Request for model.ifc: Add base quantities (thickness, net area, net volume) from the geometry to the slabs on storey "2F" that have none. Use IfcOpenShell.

First a look at what the model holds.

```python
import ifcopenshell
import ifcopenshell.util.element
import ifcopenshell.util.unit

model = ifcopenshell.open("model.ifc")
print(model.schema)
for unit_type in ("LENGTHUNIT", "AREAUNIT", "VOLUMEUNIT"):
    print(unit_type, ifcopenshell.util.unit.calculate_unit_scale(model, unit_type))
storey = next(s for s in model.by_type("IfcBuildingStorey") if s.Name == "2F")
slabs = [e for e in ifcopenshell.util.element.get_decomposition(storey) if e.is_a("IfcSlab")]
for e in sorted(slabs, key=lambda e: e.id()):
    print(e.id(), e.is_a(), e.Name, list(ifcopenshell.util.element.get_psets(e, qtos_only=True)), sep=" | ")
```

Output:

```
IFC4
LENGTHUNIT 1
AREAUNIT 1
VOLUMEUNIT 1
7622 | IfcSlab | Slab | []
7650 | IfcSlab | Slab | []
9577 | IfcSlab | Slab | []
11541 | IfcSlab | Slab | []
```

```python
import ifcopenshell
import ifcopenshell.api.pset
import ifcopenshell.geom
import ifcopenshell.util.element
import ifcopenshell.util.shape
import ifcopenshell.util.unit

model = ifcopenshell.open("model.ifc")
unit_scale = ifcopenshell.util.unit.calculate_unit_scale(model)
area_scale = ifcopenshell.util.unit.calculate_unit_scale(model, "AREAUNIT")
volume_scale = ifcopenshell.util.unit.calculate_unit_scale(model, "VOLUMEUNIT")
settings = ifcopenshell.geom.settings()

storey = next(s for s in model.by_type("IfcBuildingStorey") if s.Name == "2F")
slabs = [e for e in ifcopenshell.util.element.get_decomposition(storey) if e.is_a("IfcSlab")]

for e in sorted(slabs, key=lambda e: e.id()):
    if ifcopenshell.util.element.get_psets(e, qtos_only=True, should_inherit=False):
        continue
    # Geometry comes back in metres, in the element's own axes.
    shape = ifcopenshell.geom.create_shape(settings, e)
    values = {
        "Width": ifcopenshell.util.shape.get_z(shape.geometry) / unit_scale,
        "NetArea": ifcopenshell.util.shape.get_footprint_area(shape.geometry) / area_scale,
        "NetVolume": ifcopenshell.util.shape.get_volume(shape.geometry) / volume_scale,
    }
    qto = ifcopenshell.api.pset.add_qto(model, product=e, name="Qto_SlabBaseQuantities")
    ifcopenshell.api.pset.edit_qto(model, qto=qto, properties=values)
    print(e.id(), {k: round(v, 3) for k, v in values.items()})

model.write("model_updated.ifc")
```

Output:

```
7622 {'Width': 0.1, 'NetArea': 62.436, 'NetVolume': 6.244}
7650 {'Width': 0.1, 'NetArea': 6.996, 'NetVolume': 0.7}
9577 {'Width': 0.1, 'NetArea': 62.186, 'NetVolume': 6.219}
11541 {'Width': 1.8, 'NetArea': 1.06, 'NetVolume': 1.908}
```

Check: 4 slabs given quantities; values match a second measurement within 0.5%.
